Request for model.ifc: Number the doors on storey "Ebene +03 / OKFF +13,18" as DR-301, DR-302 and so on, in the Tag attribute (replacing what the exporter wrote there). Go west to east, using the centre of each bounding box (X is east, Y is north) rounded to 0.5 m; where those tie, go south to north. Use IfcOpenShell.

First a look at what the model holds.

```python
import ifcopenshell
import ifcopenshell.util.element
import ifcopenshell.util.placement

model = ifcopenshell.open("model.ifc")
print(model.schema)
storey = next(s for s in model.by_type("IfcBuildingStorey") if s.Name == "Ebene +03 / OKFF +13,18")
doors = [e for e in ifcopenshell.util.element.get_decomposition(storey) if e.is_a("IfcDoor")]
for e in sorted(doors, key=lambda e: e.id()):
    origin = ifcopenshell.util.placement.get_local_placement(e.ObjectPlacement)[:3, 3]
    print(e.id(), e.Tag, e.Name, origin.round(2) + 0.0, sep=" | ")
```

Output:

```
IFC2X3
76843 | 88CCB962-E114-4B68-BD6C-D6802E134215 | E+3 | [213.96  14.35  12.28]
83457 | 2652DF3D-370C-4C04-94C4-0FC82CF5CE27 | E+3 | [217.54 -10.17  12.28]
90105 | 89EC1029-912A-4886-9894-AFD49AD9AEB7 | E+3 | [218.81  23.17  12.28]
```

```python
import ifcopenshell
import ifcopenshell.geom
import ifcopenshell.util.element
import ifcopenshell.util.shape

model = ifcopenshell.open("model.ifc")
settings = ifcopenshell.geom.settings()
settings.set("use-world-coords", True)


def centre(element):
    shape = ifcopenshell.geom.create_shape(settings, element)
    return ifcopenshell.util.shape.get_bbox_centroid(shape.geometry)


storey = next(s for s in model.by_type("IfcBuildingStorey") if s.Name == "Ebene +03 / OKFF +13,18")
doors = [e for e in ifcopenshell.util.element.get_decomposition(storey) if e.is_a("IfcDoor")]

# Insertion points can sit at a corner or the storey origin, so sort by the geometry (in metres).
centres = {e: centre(e) for e in doors}
doors.sort(key=lambda e: (round(centres[e][0] / 0.5), centres[e][1]))

for i, e in enumerate(doors, start=1):
    number = f"DR-3{i:02d}"
    e.Tag = number
    print(e.id(), number)

model.write("model_edited.ifc")
```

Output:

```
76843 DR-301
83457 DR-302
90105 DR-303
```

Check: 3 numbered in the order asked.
